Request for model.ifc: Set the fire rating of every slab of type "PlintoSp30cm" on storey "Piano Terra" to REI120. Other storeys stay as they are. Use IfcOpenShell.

First a look at what the model holds.

```python
import ifcopenshell
import ifcopenshell.util.element

model = ifcopenshell.open("model.ifc")
print(model.schema)
storey = next(s for s in model.by_type("IfcBuildingStorey") if s.Name == "Piano Terra")
slabs = [e for e in ifcopenshell.util.element.get_decomposition(storey) if e.is_a("IfcSlab")]
seen = {}
for e in slabs:
    element_type = ifcopenshell.util.element.get_type(e)
    key = (element_type.Name if element_type != e and element_type else None, ifcopenshell.util.element.get_pset(e, "Pset_SlabCommon", "FireRating"))
    seen[key] = seen.get(key, 0) + 1
for (name, value), count in sorted(seen.items(), key=str):
    print(count, "x", name, "|", value)
```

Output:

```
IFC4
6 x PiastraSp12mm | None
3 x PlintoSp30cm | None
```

```python
import ifcopenshell
import ifcopenshell.api.pset
import ifcopenshell.util.element

model = ifcopenshell.open("model.ifc")

storey = next(s for s in model.by_type("IfcBuildingStorey") if s.Name == "Piano Terra")
slabs = [e for e in ifcopenshell.util.element.get_decomposition(storey) if e.is_a("IfcSlab")]

count = 0
for e in slabs:
    element_type = ifcopenshell.util.element.get_type(e)
    if element_type in (None, e) or element_type.Name != "PlintoSp30cm":
        continue
    # add_pset returns the element's existing set when there is one.
    pset = ifcopenshell.api.pset.add_pset(model, product=e, name="Pset_SlabCommon")
    ifcopenshell.api.pset.edit_pset(model, pset=pset, properties={"FireRating": "REI120"})
    count += 1

print(count, "slabs updated")

model.write("model_updated.ifc")
```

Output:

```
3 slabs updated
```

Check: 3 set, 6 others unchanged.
